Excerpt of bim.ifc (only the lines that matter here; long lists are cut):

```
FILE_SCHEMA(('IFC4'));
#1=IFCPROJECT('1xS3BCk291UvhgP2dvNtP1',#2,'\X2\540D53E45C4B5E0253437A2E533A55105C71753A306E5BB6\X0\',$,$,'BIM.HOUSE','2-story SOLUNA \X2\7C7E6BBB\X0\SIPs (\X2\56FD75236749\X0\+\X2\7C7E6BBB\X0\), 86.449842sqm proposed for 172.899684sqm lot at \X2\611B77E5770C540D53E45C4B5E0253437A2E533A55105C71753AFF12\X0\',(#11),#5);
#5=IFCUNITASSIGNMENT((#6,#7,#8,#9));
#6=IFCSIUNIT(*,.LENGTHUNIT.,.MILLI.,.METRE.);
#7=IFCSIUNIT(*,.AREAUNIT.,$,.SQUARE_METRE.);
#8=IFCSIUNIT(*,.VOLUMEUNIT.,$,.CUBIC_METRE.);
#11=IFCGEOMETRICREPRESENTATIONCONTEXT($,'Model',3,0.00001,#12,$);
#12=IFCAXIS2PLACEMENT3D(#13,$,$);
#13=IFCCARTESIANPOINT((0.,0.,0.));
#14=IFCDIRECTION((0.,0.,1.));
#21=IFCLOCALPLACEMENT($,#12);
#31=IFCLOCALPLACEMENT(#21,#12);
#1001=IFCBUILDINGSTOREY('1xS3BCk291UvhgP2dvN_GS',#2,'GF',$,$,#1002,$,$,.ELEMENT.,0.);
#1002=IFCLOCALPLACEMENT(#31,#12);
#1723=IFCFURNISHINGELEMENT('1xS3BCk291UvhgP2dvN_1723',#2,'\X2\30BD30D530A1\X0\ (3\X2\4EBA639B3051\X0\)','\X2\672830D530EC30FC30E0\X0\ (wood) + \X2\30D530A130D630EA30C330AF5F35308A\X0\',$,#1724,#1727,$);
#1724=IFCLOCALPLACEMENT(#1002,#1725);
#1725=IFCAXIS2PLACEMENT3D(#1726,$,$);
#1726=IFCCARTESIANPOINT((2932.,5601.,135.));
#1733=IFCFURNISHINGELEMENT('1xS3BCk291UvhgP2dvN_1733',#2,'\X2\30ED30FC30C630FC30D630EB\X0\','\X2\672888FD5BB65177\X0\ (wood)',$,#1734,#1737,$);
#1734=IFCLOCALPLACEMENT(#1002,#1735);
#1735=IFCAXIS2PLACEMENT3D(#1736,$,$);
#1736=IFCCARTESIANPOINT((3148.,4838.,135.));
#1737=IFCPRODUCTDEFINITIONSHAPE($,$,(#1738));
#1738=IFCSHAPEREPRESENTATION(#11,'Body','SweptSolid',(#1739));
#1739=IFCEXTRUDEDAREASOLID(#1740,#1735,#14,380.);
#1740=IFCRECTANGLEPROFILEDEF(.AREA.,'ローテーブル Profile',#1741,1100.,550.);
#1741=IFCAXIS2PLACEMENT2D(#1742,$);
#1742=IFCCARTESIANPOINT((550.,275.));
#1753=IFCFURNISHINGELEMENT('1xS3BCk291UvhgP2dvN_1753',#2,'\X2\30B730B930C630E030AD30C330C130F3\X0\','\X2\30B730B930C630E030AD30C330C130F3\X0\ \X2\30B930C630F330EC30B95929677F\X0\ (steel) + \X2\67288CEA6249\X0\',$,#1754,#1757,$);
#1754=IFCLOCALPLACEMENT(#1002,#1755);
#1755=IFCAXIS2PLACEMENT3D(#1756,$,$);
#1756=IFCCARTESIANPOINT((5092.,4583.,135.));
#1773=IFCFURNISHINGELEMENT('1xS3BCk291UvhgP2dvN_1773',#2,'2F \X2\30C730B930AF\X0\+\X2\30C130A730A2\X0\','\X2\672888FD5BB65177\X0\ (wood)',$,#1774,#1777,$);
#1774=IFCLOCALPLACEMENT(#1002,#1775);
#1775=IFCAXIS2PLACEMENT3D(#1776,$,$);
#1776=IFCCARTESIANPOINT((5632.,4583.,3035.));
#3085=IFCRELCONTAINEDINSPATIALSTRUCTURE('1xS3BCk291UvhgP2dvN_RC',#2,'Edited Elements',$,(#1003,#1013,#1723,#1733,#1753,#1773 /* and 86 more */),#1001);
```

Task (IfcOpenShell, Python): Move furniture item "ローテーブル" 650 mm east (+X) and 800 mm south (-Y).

```python
import ifcopenshell
import ifcopenshell.api.geometry
import ifcopenshell.util.placement
import ifcopenshell.util.unit

model = ifcopenshell.open("bim.ifc")
unit_scale = ifcopenshell.util.unit.calculate_unit_scale(model)

item = model.by_guid("1xS3BCk291UvhgP2dvN_1733")
matrix = ifcopenshell.util.placement.get_local_placement(item.ObjectPlacement)
matrix[0, 3] += 0.65 / unit_scale
matrix[1, 3] -= 0.8 / unit_scale
ifcopenshell.api.geometry.edit_object_placement(model, product=item, matrix=matrix, is_si=False)

print(ifcopenshell.util.placement.get_local_placement(item.ObjectPlacement).round(3) + 0.0)

model.write("bim_updated.ifc")
```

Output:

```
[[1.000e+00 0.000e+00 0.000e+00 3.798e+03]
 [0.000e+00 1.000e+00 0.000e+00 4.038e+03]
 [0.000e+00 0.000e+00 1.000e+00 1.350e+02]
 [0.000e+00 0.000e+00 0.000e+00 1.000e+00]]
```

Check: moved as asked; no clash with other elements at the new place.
